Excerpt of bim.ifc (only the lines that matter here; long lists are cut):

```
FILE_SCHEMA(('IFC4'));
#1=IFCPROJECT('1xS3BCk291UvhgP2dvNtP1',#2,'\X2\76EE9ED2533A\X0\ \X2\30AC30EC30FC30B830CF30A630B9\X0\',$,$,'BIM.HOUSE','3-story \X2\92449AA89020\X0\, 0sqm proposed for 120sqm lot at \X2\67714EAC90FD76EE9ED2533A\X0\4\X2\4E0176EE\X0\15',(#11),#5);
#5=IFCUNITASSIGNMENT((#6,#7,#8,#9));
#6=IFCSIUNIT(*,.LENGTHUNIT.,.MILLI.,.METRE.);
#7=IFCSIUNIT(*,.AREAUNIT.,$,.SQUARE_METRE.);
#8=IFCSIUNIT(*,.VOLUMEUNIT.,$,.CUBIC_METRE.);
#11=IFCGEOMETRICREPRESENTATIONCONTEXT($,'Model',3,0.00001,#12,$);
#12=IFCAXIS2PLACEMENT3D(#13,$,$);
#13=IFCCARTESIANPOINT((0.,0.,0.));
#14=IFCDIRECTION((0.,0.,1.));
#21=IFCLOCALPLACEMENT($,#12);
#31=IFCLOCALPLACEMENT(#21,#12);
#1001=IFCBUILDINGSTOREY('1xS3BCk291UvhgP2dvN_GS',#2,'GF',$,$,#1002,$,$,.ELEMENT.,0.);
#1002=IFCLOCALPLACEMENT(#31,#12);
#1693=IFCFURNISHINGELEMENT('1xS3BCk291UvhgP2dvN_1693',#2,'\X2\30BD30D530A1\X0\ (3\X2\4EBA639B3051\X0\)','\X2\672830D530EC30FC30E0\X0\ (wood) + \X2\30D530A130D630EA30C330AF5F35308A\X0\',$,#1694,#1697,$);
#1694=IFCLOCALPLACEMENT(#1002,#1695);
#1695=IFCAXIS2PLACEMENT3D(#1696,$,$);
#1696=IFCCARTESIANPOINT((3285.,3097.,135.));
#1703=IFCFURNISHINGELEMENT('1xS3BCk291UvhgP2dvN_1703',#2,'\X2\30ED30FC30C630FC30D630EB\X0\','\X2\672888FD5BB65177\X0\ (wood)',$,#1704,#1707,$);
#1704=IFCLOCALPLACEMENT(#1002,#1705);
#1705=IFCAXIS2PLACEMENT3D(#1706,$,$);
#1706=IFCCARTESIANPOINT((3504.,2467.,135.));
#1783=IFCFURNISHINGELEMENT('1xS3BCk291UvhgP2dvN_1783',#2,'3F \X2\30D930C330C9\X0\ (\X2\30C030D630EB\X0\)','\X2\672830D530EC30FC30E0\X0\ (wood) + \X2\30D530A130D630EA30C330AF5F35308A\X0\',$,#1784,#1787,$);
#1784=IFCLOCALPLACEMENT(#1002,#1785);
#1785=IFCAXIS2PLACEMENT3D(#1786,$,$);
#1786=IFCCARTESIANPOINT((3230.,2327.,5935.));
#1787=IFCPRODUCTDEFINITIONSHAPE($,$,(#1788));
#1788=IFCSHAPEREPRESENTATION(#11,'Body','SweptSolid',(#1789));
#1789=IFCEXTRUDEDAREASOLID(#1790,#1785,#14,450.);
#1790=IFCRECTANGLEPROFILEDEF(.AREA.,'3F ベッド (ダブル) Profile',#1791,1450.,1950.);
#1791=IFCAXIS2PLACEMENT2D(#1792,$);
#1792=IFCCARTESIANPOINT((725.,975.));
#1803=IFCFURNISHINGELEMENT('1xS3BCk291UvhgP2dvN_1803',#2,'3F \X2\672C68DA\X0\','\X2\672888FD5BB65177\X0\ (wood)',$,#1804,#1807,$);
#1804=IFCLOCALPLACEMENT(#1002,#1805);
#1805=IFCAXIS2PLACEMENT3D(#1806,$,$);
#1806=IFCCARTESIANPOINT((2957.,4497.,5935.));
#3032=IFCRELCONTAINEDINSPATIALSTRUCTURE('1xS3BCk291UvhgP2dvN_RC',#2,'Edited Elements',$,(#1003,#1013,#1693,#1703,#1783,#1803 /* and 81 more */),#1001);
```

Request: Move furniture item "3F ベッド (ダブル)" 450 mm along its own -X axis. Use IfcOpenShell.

```python
import ifcopenshell
import ifcopenshell.api.geometry
import ifcopenshell.util.placement
import ifcopenshell.util.unit

model = ifcopenshell.open("bim.ifc")
unit_scale = ifcopenshell.util.unit.calculate_unit_scale(model)

item = model.by_guid("1xS3BCk291UvhgP2dvN_1783")
matrix = ifcopenshell.util.placement.get_local_placement(item.ObjectPlacement)
matrix[:3, 3] -= matrix[:3, 0] * 0.45 / unit_scale
ifcopenshell.api.geometry.edit_object_placement(model, product=item, matrix=matrix, is_si=False)

print(ifcopenshell.util.placement.get_local_placement(item.ObjectPlacement).round(3) + 0.0)

model.write("bim-out.ifc")
```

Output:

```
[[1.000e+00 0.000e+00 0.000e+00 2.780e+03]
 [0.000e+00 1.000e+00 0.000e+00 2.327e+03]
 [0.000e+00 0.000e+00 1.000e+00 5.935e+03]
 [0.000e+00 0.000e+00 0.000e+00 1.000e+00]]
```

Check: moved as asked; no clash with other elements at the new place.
